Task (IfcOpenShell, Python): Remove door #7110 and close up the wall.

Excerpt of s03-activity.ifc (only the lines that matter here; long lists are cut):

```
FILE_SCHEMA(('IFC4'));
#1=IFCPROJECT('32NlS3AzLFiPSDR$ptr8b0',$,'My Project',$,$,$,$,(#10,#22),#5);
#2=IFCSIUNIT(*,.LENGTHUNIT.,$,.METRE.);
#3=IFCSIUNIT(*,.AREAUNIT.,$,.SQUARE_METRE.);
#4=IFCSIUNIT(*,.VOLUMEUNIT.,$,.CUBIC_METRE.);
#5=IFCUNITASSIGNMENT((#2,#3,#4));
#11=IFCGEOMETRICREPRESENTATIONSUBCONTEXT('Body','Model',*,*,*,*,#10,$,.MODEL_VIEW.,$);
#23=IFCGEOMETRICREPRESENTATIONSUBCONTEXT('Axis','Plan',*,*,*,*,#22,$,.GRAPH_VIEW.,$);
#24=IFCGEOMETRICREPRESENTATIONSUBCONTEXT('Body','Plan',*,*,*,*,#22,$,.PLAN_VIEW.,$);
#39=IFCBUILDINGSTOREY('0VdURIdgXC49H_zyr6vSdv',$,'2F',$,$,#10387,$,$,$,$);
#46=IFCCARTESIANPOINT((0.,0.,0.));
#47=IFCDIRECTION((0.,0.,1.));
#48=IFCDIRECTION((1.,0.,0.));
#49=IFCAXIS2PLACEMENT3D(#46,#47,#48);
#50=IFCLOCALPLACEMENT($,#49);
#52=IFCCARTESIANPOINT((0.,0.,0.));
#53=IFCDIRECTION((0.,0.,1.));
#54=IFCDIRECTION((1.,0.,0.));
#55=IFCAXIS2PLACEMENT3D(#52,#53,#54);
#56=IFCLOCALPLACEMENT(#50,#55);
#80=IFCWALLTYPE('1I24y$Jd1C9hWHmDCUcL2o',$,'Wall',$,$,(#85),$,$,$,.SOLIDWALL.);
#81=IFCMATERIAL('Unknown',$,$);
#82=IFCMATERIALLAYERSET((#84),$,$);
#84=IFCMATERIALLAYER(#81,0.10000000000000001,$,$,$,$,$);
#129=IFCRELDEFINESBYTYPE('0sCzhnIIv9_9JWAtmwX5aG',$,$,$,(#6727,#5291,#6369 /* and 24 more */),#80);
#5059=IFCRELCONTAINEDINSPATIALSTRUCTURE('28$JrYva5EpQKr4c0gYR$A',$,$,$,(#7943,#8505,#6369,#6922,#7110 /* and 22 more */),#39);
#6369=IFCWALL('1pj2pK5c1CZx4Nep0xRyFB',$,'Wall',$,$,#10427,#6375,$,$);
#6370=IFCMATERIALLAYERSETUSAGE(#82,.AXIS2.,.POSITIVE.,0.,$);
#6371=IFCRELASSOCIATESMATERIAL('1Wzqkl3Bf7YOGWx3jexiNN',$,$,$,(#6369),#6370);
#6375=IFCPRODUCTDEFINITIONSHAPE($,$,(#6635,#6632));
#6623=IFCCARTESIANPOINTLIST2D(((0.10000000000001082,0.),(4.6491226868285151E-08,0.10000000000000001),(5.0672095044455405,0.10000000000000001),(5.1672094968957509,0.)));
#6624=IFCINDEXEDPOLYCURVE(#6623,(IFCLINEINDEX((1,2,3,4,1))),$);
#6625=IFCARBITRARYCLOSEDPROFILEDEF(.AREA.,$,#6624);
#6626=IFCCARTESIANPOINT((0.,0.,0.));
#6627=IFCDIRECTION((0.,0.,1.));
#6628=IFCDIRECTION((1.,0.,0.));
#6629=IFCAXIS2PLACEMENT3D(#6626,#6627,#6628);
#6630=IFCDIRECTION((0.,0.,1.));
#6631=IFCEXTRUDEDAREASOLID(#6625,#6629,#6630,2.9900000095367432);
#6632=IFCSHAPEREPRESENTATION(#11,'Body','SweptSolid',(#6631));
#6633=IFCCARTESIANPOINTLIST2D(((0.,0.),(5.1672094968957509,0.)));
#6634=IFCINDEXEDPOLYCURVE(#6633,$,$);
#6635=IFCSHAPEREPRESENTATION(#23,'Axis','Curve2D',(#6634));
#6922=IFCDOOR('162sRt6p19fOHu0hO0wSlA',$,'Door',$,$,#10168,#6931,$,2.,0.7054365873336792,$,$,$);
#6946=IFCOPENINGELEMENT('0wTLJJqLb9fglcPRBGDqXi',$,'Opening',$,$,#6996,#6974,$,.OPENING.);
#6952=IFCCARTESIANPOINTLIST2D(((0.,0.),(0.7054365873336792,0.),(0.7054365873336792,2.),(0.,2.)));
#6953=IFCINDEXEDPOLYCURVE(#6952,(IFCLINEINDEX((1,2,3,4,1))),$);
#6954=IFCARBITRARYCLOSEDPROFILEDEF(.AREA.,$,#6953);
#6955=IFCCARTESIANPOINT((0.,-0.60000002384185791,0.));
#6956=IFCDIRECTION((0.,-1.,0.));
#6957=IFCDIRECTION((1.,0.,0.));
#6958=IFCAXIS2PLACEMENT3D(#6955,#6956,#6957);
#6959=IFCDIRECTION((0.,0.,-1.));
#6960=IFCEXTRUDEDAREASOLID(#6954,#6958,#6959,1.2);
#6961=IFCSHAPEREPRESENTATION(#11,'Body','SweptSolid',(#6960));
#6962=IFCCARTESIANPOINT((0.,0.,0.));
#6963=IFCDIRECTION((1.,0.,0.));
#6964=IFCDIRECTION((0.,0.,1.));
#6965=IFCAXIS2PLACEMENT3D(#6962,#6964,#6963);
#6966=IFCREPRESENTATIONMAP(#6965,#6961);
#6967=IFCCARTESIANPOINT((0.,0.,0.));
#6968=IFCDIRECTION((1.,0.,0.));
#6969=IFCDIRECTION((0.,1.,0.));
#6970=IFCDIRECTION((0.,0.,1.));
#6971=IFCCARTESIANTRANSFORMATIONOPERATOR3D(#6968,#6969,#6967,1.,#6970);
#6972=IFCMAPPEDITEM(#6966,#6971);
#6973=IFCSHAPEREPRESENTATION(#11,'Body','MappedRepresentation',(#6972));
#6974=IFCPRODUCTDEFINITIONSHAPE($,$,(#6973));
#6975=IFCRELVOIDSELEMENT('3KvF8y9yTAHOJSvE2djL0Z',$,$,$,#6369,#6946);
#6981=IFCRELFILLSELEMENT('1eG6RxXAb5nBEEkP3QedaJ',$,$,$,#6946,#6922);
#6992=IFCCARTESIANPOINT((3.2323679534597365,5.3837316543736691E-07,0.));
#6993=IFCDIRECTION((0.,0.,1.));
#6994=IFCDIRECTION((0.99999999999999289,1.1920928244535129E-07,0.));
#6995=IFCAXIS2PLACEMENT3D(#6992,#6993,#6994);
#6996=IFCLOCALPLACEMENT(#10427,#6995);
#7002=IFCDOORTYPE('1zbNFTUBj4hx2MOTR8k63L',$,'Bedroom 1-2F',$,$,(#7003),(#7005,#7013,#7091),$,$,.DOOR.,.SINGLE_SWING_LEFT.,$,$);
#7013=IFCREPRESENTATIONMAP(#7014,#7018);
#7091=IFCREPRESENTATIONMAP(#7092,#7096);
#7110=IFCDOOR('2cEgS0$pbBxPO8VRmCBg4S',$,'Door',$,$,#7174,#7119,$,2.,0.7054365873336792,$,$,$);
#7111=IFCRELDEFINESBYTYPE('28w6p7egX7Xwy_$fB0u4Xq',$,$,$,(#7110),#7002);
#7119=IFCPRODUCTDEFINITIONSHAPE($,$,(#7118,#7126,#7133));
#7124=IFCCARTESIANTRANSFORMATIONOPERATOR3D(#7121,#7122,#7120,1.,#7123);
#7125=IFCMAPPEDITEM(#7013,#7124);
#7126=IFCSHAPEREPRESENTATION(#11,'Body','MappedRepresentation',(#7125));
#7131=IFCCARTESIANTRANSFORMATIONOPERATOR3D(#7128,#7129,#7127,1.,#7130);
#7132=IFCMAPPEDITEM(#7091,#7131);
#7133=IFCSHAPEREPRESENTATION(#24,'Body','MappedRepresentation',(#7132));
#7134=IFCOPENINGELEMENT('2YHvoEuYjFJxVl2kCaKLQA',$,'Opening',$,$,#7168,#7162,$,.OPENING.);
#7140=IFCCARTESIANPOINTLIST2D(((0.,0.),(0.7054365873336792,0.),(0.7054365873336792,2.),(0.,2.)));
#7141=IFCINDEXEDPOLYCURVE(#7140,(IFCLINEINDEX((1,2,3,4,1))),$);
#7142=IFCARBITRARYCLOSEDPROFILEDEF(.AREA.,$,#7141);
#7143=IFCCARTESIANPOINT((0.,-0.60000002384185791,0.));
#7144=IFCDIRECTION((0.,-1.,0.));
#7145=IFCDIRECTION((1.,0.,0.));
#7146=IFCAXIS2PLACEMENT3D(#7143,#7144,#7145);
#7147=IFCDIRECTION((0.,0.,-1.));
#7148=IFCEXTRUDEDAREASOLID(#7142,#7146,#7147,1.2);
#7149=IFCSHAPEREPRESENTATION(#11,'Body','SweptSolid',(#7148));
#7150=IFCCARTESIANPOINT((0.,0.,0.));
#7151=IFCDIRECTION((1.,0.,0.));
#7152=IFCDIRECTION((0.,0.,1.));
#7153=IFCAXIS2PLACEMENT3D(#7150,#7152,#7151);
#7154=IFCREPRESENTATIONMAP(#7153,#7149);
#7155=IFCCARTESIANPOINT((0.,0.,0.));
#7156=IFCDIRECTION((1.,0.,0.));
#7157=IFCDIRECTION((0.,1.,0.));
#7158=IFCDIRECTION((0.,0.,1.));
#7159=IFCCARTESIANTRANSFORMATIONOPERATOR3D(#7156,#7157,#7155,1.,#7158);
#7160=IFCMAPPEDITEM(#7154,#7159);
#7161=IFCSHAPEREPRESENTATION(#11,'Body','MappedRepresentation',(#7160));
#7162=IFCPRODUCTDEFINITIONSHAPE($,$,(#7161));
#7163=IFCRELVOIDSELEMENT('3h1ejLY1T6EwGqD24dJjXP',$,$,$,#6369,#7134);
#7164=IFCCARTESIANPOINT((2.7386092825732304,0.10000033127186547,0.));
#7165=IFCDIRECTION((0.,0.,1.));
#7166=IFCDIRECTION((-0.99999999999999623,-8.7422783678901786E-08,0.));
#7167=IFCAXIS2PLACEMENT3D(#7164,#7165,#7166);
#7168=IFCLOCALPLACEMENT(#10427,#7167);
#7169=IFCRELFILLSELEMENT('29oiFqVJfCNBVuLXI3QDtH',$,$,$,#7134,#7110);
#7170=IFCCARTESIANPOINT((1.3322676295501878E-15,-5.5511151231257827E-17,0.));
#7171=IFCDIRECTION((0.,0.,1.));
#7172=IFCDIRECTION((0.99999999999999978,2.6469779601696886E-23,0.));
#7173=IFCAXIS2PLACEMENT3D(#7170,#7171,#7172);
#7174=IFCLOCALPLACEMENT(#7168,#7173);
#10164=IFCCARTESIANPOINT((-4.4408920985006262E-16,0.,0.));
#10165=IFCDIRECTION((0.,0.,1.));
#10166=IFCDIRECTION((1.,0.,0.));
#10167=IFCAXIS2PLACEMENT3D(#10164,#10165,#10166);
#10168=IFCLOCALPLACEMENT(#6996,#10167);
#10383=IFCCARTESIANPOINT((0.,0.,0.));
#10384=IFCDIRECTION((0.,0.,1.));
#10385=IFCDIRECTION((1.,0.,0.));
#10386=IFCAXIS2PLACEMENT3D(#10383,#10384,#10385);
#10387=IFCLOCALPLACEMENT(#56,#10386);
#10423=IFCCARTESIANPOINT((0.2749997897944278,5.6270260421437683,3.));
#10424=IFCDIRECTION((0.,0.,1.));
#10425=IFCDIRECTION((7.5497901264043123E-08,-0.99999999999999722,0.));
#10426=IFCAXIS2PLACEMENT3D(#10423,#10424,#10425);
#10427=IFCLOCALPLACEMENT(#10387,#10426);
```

```python
import ifcopenshell
import ifcopenshell.api.feature
import ifcopenshell.api.root
import ifcopenshell.geom
import ifcopenshell.util.shape

model = ifcopenshell.open("s03-activity.ifc")
settings = ifcopenshell.geom.settings()


def volume(element):
    """Net volume in cubic metres, openings subtracted."""
    shape = ifcopenshell.geom.create_shape(settings, element)
    return ifcopenshell.util.shape.get_volume(shape.geometry)


door = model.by_guid("2cEgS0$pbBxPO8VRmCBg4S")
opening = door.FillsVoids[0].RelatingOpeningElement
wall = opening.VoidsElements[0].RelatingBuildingElement
before = volume(wall)

ifcopenshell.api.root.remove_product(model, product=door)
ifcopenshell.api.feature.remove_feature(model, feature=opening)

after = volume(wall)

print(f"wall volume {before:.3f} -> {after:.3f} m3")

model.write("s03-activity_edited.ifc")
```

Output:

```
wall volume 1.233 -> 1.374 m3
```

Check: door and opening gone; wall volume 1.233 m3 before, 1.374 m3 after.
